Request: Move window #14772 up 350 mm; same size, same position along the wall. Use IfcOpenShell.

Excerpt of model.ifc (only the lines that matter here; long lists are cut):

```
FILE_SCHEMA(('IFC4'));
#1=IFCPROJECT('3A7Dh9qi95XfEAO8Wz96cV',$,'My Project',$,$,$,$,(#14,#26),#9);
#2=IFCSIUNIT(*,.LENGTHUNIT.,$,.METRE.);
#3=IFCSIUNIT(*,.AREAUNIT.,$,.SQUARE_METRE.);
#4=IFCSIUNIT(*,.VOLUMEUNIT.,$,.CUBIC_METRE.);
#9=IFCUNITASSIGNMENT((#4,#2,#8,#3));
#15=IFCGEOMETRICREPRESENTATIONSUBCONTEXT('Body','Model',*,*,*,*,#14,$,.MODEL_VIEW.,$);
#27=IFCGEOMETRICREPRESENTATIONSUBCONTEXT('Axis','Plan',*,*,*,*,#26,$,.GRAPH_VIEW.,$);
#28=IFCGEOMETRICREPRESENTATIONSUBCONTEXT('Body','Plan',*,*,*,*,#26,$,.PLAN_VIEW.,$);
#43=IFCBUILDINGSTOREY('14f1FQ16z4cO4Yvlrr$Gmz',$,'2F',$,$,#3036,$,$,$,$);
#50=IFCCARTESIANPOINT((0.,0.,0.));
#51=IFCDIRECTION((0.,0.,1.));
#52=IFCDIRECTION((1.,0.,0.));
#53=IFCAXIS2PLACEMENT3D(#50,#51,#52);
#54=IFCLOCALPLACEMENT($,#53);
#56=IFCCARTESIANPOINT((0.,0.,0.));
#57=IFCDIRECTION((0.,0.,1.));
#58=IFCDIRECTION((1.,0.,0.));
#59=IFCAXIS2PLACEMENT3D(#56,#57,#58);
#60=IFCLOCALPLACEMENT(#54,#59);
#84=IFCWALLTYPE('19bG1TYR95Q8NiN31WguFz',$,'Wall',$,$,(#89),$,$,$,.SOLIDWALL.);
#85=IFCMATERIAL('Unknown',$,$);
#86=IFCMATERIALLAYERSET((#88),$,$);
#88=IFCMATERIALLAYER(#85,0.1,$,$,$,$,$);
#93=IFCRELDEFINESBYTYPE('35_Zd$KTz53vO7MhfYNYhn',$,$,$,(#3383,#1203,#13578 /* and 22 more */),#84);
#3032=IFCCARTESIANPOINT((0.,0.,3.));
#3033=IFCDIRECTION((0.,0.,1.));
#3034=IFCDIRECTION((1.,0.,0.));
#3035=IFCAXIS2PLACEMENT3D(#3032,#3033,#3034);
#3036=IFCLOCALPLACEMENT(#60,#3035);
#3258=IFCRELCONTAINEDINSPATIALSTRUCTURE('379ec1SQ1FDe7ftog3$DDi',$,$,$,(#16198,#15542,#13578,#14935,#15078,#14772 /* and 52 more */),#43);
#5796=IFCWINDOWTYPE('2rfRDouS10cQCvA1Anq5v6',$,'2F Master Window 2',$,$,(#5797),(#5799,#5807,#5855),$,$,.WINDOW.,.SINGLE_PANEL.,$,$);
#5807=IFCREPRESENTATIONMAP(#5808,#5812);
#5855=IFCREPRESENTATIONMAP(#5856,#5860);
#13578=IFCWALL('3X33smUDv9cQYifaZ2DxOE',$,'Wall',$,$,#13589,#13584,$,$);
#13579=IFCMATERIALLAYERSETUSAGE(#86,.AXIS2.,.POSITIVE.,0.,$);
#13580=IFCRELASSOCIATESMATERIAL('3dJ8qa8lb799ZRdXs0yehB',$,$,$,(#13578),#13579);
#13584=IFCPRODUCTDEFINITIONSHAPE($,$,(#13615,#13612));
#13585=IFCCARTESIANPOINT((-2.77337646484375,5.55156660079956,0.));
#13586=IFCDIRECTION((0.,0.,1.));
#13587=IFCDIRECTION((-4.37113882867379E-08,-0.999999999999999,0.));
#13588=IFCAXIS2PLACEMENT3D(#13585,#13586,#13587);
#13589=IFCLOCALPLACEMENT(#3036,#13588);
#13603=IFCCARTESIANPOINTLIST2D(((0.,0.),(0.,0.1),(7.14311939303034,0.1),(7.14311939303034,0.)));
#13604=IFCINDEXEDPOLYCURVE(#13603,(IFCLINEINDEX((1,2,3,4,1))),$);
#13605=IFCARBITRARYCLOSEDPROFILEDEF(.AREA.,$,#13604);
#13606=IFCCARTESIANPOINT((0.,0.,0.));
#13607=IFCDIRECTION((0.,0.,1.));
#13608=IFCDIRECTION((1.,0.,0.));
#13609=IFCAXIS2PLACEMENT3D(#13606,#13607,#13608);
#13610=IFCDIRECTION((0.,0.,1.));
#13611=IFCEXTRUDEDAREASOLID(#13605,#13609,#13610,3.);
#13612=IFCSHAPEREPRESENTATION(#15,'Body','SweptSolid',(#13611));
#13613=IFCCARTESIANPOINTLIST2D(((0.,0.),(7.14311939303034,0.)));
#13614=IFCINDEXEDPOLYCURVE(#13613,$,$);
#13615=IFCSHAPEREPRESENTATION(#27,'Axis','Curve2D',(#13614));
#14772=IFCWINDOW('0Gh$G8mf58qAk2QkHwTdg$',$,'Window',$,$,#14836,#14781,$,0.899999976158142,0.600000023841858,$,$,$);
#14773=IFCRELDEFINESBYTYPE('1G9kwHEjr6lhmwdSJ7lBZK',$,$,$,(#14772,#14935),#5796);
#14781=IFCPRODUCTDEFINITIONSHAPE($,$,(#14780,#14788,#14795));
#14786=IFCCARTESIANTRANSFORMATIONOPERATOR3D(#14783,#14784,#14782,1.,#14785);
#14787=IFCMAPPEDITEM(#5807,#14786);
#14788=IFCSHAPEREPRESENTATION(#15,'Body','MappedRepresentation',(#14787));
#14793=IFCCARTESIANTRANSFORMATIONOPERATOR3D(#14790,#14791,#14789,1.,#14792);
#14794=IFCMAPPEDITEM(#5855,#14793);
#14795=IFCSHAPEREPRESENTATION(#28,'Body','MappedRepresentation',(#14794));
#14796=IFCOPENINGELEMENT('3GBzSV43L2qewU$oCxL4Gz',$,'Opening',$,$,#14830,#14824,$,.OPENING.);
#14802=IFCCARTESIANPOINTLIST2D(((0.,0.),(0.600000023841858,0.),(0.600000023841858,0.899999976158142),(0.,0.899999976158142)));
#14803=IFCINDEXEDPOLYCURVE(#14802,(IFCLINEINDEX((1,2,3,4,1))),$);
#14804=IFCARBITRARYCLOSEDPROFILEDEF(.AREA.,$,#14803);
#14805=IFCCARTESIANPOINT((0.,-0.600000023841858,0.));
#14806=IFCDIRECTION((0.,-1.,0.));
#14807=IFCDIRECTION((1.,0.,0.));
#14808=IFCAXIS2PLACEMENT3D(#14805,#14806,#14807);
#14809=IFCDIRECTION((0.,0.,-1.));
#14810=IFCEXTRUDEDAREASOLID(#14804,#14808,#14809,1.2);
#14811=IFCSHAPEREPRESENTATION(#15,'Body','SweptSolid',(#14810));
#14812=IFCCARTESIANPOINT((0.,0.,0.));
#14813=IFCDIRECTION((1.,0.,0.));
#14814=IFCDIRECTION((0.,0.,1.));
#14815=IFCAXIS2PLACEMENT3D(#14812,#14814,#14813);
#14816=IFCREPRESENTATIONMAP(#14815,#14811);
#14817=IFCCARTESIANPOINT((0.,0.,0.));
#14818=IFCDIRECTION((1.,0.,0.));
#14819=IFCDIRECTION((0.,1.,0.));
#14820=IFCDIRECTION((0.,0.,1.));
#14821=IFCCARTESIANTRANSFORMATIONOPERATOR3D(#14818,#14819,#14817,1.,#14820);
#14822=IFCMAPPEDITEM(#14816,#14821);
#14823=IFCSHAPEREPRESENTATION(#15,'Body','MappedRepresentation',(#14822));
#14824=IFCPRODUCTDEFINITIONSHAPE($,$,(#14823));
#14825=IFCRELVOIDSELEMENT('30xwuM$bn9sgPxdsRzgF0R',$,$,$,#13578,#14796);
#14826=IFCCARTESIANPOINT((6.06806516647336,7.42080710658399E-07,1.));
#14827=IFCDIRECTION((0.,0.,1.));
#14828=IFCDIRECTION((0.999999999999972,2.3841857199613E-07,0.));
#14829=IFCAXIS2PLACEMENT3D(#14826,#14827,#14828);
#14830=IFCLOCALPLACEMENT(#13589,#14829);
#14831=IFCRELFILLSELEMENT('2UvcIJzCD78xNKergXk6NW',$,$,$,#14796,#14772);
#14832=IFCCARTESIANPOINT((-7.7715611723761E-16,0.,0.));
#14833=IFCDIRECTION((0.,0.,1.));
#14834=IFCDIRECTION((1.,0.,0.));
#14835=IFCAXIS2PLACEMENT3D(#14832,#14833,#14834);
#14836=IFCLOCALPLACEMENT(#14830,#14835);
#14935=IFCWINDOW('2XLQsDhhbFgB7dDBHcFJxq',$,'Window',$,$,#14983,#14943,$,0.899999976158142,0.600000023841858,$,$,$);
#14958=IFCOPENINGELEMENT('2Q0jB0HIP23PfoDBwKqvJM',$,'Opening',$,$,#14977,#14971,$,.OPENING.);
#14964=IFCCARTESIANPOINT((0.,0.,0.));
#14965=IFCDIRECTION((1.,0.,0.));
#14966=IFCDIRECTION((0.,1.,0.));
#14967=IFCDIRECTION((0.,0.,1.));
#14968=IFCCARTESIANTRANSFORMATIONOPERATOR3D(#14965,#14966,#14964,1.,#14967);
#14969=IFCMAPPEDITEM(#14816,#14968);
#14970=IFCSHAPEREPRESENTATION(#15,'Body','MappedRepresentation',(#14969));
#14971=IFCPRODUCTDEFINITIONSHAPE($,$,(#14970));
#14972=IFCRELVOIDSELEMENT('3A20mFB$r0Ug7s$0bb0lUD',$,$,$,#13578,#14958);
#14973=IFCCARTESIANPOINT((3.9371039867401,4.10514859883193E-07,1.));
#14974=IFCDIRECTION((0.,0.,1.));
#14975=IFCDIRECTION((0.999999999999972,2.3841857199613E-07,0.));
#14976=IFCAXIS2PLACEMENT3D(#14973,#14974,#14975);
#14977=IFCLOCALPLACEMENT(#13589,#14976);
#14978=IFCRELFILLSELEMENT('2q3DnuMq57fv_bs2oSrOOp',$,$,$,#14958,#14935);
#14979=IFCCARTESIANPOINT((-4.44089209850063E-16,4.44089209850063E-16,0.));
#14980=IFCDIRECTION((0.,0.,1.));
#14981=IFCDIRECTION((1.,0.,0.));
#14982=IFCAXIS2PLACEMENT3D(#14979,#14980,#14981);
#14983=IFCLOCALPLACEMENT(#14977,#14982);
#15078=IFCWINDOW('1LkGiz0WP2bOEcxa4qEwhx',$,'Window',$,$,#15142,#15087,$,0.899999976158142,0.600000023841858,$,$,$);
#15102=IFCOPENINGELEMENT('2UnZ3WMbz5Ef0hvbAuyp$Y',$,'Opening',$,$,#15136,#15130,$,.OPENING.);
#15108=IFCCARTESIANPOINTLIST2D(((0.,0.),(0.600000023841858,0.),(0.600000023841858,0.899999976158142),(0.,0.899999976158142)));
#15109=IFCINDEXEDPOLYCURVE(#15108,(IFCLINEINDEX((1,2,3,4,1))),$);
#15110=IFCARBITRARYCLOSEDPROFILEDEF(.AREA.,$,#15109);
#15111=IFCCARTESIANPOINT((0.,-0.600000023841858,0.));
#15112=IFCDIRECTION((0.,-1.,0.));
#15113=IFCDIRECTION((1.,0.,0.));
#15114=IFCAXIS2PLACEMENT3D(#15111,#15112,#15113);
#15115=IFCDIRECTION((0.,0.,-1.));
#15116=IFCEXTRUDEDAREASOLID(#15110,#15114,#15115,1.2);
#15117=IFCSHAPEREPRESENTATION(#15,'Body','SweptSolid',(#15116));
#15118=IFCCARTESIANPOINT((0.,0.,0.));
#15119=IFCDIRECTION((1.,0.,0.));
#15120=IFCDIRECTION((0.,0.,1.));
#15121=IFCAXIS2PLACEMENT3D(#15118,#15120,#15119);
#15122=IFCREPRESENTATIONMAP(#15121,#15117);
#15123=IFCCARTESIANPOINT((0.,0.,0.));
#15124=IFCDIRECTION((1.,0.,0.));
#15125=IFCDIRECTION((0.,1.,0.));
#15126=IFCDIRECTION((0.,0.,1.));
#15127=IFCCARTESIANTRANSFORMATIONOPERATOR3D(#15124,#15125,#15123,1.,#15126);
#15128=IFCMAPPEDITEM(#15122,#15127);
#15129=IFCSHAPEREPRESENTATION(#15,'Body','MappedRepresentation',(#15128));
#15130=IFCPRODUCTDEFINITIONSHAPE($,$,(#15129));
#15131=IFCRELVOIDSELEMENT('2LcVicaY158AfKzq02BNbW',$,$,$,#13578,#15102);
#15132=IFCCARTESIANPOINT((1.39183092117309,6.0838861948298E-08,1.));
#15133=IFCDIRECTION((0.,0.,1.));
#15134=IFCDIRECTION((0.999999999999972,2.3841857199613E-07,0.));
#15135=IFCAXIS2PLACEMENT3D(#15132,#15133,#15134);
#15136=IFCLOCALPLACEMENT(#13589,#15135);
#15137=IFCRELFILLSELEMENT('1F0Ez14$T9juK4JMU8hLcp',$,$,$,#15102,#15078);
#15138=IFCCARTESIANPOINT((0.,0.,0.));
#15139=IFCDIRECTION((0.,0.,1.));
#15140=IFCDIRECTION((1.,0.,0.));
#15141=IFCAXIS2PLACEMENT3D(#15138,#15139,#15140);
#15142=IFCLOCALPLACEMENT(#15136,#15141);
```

```python
import numpy as np
import ifcopenshell
import ifcopenshell.api.geometry
import ifcopenshell.util.placement
import ifcopenshell.util.unit

model = ifcopenshell.open("model.ifc")
unit_scale = ifcopenshell.util.unit.calculate_unit_scale(model)

window = model.by_id(14772)
opening = window.FillsVoids[0].RelatingOpeningElement
dz = 0.35 / unit_scale

shift = np.array([0.0, 0.0, dz])
# The window is placed relative to its opening, so it follows when the opening moves.
matrix = ifcopenshell.util.placement.get_local_placement(opening.ObjectPlacement)
matrix[:3, 3] += shift
ifcopenshell.api.geometry.edit_object_placement(
    model, product=opening, matrix=matrix, is_si=False, should_transform_children=True
)

print(f"moved by {dz * unit_scale:+.3f} m")

model.write("model_edited.ifc")
```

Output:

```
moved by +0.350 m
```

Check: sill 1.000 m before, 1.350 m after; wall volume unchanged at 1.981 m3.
